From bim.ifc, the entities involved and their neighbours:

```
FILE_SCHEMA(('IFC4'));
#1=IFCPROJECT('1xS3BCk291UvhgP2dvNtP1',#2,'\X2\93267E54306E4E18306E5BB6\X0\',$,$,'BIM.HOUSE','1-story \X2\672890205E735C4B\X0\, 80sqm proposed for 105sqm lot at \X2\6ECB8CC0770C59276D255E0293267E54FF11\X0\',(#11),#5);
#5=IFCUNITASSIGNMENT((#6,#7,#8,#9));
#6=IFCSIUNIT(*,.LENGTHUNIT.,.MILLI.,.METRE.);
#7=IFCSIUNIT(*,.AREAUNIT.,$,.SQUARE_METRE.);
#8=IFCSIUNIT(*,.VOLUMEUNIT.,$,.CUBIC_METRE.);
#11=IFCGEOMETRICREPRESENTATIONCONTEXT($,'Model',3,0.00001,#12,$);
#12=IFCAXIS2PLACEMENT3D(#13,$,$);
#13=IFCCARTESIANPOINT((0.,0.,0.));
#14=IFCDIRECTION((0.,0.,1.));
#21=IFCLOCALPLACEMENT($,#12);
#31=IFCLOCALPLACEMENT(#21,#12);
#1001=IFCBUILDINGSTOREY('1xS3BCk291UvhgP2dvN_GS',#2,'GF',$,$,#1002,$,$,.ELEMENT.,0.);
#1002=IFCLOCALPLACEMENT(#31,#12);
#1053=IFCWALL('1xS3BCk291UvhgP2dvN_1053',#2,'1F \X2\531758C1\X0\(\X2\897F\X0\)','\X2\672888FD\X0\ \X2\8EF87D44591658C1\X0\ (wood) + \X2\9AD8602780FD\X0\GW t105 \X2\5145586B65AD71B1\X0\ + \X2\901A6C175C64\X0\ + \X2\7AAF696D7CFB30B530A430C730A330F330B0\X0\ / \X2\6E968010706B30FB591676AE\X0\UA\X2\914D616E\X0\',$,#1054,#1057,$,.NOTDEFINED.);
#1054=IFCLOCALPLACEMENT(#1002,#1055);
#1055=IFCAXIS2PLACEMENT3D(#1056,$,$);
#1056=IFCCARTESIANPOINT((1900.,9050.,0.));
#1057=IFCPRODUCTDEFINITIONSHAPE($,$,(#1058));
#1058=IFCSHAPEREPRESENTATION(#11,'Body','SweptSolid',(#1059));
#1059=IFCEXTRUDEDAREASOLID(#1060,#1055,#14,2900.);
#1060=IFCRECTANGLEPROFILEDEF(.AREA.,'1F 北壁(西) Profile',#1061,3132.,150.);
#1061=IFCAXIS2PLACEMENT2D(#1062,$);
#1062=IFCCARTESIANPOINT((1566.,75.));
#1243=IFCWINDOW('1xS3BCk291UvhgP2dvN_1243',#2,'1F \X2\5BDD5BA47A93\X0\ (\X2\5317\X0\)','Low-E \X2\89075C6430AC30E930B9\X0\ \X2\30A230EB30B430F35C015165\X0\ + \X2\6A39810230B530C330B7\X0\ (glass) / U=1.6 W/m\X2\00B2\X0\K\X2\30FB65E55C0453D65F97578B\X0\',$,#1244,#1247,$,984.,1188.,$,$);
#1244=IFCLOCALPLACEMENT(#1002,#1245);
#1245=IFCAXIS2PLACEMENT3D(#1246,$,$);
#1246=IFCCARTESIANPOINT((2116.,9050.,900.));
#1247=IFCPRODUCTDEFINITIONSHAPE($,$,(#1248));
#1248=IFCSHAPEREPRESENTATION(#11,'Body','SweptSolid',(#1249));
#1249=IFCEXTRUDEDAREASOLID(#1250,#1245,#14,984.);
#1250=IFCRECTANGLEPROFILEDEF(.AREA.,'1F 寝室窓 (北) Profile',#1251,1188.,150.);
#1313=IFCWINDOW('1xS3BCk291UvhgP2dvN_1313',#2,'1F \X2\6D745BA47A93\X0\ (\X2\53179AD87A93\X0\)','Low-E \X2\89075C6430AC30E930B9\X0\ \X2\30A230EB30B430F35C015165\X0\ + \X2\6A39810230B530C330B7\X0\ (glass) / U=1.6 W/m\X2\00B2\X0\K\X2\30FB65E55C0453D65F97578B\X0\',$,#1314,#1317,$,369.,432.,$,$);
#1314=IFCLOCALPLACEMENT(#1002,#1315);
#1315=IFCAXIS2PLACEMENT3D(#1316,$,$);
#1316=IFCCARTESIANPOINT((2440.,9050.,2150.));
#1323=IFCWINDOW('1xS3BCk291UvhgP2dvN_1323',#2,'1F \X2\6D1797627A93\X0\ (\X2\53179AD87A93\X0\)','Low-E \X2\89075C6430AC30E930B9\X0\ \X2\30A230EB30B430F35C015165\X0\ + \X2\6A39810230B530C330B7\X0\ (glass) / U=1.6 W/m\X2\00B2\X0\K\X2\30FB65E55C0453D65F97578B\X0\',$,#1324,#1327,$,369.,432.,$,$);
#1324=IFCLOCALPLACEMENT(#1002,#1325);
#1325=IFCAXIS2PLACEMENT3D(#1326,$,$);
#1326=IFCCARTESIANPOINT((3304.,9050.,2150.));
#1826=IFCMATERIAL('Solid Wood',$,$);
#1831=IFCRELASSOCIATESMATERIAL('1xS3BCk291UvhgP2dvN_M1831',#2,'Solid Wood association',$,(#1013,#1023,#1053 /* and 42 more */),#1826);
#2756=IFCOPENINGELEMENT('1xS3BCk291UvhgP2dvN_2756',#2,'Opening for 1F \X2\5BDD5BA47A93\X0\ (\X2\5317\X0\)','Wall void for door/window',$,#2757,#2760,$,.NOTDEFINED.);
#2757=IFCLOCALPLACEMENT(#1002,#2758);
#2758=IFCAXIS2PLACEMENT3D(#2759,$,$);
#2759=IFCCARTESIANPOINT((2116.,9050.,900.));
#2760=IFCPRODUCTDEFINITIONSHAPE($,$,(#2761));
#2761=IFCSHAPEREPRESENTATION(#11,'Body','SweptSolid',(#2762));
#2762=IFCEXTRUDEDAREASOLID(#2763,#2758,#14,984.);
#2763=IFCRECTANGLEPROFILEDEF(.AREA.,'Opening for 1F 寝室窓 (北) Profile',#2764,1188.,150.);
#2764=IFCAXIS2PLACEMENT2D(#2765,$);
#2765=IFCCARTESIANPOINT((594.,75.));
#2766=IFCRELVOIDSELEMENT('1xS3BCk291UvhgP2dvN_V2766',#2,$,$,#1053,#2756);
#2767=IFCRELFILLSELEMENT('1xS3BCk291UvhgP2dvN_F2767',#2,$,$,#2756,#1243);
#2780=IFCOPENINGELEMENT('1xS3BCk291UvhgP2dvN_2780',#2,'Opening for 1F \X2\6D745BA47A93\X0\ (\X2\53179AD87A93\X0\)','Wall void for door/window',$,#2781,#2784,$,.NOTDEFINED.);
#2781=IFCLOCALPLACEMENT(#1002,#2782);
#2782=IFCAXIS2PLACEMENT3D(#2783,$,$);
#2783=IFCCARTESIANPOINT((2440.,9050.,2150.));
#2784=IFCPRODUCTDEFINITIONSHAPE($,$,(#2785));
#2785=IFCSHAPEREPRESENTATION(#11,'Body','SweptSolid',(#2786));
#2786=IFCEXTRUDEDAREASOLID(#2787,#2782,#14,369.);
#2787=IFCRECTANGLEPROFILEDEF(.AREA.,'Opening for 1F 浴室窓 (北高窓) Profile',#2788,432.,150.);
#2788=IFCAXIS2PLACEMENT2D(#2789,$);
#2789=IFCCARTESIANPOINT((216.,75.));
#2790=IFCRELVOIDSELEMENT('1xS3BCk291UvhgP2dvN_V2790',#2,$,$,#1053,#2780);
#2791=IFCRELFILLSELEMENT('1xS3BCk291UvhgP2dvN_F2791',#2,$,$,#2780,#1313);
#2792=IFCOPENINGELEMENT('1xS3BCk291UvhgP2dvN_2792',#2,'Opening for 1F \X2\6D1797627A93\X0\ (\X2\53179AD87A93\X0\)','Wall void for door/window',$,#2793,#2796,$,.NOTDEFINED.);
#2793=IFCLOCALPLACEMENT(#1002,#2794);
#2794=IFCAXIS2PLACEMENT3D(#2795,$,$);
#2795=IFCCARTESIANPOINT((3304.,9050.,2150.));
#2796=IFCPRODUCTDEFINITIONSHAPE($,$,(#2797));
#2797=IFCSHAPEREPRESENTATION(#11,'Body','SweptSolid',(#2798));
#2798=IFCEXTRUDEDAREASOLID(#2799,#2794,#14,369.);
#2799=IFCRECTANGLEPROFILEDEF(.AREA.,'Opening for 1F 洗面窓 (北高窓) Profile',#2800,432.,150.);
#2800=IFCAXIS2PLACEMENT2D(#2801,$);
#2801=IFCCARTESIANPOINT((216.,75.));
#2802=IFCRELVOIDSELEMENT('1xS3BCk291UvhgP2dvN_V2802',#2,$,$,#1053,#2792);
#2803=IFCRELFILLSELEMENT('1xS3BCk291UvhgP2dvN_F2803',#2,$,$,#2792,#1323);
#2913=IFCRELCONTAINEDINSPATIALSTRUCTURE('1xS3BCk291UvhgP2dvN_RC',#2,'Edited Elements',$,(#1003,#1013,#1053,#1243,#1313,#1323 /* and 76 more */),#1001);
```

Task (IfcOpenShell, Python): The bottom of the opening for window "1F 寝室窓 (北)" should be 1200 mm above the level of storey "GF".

```python
import numpy as np
import ifcopenshell
import ifcopenshell.api.geometry
import ifcopenshell.geom
import ifcopenshell.util.element
import ifcopenshell.util.placement
import ifcopenshell.util.shape
import ifcopenshell.util.unit

model = ifcopenshell.open("bim.ifc")
unit_scale = ifcopenshell.util.unit.calculate_unit_scale(model)

window = model.by_guid("1xS3BCk291UvhgP2dvN_1243")
opening = window.FillsVoids[0].RelatingOpeningElement
storey = ifcopenshell.util.element.get_container(window, ifc_class="IfcBuildingStorey")
level = ifcopenshell.util.placement.get_local_placement(storey.ObjectPlacement)[2, 3]

# The opening's origin need not be at the sill, so measure its lowest point.
shape = ifcopenshell.geom.create_shape(ifcopenshell.geom.settings(), opening)
bottom = ifcopenshell.util.shape.get_shape_bottom_elevation(shape, shape.geometry) / unit_scale
dz = level + 1.2 / unit_scale - bottom

shift = np.array([0.0, 0.0, dz])
# The window is not placed relative to its opening, so move both.
for product in (opening, window):
    matrix = ifcopenshell.util.placement.get_local_placement(product.ObjectPlacement)
    matrix[:3, 3] += shift
    ifcopenshell.api.geometry.edit_object_placement(model, product=product, matrix=matrix, is_si=False)

print(f"moved by {dz * unit_scale:+.3f} m")

model.write("bim_v2.ifc")
```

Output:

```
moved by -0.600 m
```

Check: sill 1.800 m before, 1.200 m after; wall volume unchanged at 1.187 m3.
